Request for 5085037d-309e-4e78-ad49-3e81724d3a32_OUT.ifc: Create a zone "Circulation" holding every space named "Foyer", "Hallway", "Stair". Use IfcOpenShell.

First a look at what the model holds.

```python
import ifcopenshell

model = ifcopenshell.open("5085037d-309e-4e78-ad49-3e81724d3a32_OUT.ifc")
print(model.schema)
seen = {}
for space in model.by_type("IfcSpace"):
    seen[space.LongName] = seen.get(space.LongName, 0) + 1
for name, count in sorted(seen.items(), key=str):
    print(count, "x", name)
print("zones:", [z.Name for z in model.by_type("IfcZone")][:20])
```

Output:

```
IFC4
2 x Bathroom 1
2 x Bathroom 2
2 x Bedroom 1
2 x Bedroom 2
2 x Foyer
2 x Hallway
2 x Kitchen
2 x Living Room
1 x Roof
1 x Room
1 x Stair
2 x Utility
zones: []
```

```python
import ifcopenshell
import ifcopenshell.api.group
import ifcopenshell.api.root

model = ifcopenshell.open("5085037d-309e-4e78-ad49-3e81724d3a32_OUT.ifc")

names = {"Foyer", "Hallway", "Stair"}
spaces = [s for s in model.by_type("IfcSpace") if s.LongName in names]

zone = ifcopenshell.api.root.create_entity(model, ifc_class="IfcZone", name="Circulation")
ifcopenshell.api.group.assign_group(model, products=spaces, group=zone)
print(len(spaces), "spaces in", zone.Name)

model.write("5085037d-309e-4e78-ad49-3e81724d3a32_OUT_rev.ifc")
```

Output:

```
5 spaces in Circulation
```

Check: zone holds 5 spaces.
